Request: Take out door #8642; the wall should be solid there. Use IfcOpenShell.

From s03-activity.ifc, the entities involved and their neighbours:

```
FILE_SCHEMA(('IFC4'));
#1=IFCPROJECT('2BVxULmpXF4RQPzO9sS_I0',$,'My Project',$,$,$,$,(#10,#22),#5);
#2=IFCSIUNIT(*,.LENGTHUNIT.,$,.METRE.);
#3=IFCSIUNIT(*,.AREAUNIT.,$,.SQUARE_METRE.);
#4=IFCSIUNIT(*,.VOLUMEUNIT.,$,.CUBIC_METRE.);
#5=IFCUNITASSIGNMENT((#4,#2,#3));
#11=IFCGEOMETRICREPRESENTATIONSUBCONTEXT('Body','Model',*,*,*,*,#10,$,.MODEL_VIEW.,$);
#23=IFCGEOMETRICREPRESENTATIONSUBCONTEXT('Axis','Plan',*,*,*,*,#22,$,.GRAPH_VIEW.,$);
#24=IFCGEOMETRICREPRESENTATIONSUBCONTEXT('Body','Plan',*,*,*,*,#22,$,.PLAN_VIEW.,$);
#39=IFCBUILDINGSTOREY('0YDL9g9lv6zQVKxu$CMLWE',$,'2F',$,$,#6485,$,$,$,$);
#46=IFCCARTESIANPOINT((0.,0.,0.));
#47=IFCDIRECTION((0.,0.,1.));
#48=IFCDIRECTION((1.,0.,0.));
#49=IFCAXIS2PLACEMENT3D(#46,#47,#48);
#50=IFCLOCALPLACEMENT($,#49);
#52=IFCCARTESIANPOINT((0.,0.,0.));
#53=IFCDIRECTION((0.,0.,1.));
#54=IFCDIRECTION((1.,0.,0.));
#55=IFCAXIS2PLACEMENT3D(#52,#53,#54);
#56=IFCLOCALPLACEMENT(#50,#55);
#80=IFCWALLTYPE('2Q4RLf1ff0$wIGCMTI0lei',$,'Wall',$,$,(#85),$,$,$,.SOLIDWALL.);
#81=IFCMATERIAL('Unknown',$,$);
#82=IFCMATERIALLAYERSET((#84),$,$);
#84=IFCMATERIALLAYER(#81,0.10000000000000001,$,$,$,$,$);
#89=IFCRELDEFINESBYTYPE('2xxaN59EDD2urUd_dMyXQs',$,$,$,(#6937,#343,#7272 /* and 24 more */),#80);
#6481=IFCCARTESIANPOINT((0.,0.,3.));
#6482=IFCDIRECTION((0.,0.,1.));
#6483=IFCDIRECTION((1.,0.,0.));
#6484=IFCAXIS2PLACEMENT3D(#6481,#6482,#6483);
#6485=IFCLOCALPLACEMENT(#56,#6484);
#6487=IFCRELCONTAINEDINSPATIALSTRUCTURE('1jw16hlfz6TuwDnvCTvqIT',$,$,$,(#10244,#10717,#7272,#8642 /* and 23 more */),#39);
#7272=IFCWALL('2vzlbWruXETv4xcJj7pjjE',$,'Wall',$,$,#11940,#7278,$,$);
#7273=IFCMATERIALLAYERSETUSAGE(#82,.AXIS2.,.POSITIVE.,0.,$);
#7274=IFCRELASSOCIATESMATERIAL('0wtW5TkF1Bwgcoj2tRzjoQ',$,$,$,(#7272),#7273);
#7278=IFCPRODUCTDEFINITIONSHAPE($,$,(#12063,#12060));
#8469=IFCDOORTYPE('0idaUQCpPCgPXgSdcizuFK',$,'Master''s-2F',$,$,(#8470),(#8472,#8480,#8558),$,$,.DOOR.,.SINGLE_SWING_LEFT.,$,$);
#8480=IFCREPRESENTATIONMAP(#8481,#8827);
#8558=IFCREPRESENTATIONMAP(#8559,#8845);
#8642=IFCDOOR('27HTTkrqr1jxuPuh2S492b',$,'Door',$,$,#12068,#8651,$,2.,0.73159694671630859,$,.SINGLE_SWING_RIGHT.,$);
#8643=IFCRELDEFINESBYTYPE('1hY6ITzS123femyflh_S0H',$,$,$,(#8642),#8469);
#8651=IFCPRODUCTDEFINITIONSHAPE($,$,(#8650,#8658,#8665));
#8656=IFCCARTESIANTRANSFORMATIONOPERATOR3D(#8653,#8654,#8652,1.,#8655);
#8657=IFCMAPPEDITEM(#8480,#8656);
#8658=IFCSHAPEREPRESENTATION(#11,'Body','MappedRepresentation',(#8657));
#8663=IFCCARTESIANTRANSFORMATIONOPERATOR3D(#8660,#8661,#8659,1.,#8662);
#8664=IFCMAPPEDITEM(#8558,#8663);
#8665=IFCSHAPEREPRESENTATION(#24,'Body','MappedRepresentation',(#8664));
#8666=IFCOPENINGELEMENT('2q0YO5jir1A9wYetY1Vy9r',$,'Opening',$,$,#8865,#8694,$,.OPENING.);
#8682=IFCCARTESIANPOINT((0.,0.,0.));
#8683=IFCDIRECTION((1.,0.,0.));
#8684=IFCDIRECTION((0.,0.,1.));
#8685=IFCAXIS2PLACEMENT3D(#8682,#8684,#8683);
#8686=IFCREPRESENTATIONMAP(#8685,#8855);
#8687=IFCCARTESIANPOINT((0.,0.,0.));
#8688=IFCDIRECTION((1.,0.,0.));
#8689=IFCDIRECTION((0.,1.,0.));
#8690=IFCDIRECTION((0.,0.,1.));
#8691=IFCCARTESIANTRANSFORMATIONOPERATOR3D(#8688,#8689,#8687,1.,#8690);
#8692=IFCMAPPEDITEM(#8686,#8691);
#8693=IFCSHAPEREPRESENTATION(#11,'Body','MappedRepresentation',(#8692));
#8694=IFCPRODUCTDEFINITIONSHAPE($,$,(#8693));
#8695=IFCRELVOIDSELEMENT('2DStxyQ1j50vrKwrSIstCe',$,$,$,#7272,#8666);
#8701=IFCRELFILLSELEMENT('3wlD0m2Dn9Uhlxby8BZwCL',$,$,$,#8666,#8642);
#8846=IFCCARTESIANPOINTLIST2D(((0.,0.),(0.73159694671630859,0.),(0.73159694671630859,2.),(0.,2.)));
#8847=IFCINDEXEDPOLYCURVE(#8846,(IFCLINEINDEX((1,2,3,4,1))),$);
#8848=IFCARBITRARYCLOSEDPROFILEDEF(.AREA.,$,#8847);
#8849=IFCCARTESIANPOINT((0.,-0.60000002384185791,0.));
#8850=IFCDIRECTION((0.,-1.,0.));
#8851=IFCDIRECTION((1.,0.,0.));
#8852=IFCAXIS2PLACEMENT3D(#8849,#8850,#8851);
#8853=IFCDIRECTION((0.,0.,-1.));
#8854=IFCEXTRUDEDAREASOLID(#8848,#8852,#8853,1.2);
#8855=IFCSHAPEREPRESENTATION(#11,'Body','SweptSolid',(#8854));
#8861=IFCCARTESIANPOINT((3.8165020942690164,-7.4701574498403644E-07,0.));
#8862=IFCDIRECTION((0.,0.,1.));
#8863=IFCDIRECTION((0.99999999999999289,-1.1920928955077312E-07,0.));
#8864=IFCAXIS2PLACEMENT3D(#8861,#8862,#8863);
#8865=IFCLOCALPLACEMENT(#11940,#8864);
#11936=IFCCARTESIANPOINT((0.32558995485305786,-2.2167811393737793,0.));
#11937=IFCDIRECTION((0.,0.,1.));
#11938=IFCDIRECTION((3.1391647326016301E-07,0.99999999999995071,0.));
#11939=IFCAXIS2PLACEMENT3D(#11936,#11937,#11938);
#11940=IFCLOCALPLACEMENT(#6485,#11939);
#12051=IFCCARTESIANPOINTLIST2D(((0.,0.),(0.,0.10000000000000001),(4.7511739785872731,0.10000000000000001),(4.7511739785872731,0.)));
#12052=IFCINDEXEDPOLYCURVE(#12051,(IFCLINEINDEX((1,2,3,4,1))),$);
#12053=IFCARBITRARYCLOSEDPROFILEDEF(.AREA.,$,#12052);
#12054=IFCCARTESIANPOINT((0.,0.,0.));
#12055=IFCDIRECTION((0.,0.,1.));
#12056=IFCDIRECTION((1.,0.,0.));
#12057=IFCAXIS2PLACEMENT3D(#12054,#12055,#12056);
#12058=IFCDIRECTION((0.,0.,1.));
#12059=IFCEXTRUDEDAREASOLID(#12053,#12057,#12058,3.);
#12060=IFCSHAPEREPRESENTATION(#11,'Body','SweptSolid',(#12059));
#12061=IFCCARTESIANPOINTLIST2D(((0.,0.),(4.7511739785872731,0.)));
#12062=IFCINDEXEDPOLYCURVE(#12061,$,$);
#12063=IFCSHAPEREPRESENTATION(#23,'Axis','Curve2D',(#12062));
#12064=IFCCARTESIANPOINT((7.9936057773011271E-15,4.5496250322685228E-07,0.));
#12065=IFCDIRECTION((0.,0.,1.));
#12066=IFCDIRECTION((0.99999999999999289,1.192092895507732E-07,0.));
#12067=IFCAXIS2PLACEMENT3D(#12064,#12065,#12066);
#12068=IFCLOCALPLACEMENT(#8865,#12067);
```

```python
import ifcopenshell
import ifcopenshell.api.feature
import ifcopenshell.api.root
import ifcopenshell.geom
import ifcopenshell.util.shape

model = ifcopenshell.open("s03-activity.ifc")
settings = ifcopenshell.geom.settings()


def volume(element):
    """Net volume in cubic metres, openings subtracted."""
    shape = ifcopenshell.geom.create_shape(settings, element)
    return ifcopenshell.util.shape.get_volume(shape.geometry)


door = model.by_guid("27HTTkrqr1jxuPuh2S492b")
opening = door.FillsVoids[0].RelatingOpeningElement
wall = opening.VoidsElements[0].RelatingBuildingElement
before = volume(wall)

ifcopenshell.api.root.remove_product(model, product=door)
ifcopenshell.api.feature.remove_feature(model, feature=opening)

after = volume(wall)

print(f"wall volume {before:.3f} -> {after:.3f} m3")

model.write("s03-activity-out.ifc")
```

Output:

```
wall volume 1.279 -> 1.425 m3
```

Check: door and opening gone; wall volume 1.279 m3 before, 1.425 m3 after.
